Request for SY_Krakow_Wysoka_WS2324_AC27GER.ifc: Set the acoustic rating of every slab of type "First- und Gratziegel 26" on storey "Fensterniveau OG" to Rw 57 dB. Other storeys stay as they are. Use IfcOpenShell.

First a look at what the model holds.

```python
import ifcopenshell
import ifcopenshell.util.element

model = ifcopenshell.open("SY_Krakow_Wysoka_WS2324_AC27GER.ifc")
print(model.schema)
storey = next(s for s in model.by_type("IfcBuildingStorey") if s.Name == "Fensterniveau OG")
slabs = [e for e in ifcopenshell.util.element.get_decomposition(storey) if e.is_a("IfcSlab")]
seen = {}
for e in slabs:
    element_type = ifcopenshell.util.element.get_type(e)
    key = (element_type.Name if element_type != e and element_type else None, ifcopenshell.util.element.get_pset(e, "Pset_SlabCommon", "AcousticRating"))
    seen[key] = seen.get(key, 0) + 1
for (name, value), count in sorted(seen.items(), key=str):
    print(count, "x", name, "|", value)
```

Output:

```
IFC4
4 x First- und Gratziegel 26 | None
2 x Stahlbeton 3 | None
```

```python
import ifcopenshell
import ifcopenshell.api.pset
import ifcopenshell.util.element

model = ifcopenshell.open("SY_Krakow_Wysoka_WS2324_AC27GER.ifc")

storey = next(s for s in model.by_type("IfcBuildingStorey") if s.Name == "Fensterniveau OG")
slabs = [e for e in ifcopenshell.util.element.get_decomposition(storey) if e.is_a("IfcSlab")]

count = 0
for e in slabs:
    element_type = ifcopenshell.util.element.get_type(e)
    if element_type in (None, e) or element_type.Name != "First- und Gratziegel 26":
        continue
    # add_pset returns the element's existing set when there is one.
    pset = ifcopenshell.api.pset.add_pset(model, product=e, name="Pset_SlabCommon")
    ifcopenshell.api.pset.edit_pset(model, pset=pset, properties={"AcousticRating": "Rw 57 dB"})
    count += 1

print(count, "slabs updated")

model.write("SY_Krakow_Wysoka_WS2324_AC27GER_updated.ifc")
```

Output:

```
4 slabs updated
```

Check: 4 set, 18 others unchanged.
